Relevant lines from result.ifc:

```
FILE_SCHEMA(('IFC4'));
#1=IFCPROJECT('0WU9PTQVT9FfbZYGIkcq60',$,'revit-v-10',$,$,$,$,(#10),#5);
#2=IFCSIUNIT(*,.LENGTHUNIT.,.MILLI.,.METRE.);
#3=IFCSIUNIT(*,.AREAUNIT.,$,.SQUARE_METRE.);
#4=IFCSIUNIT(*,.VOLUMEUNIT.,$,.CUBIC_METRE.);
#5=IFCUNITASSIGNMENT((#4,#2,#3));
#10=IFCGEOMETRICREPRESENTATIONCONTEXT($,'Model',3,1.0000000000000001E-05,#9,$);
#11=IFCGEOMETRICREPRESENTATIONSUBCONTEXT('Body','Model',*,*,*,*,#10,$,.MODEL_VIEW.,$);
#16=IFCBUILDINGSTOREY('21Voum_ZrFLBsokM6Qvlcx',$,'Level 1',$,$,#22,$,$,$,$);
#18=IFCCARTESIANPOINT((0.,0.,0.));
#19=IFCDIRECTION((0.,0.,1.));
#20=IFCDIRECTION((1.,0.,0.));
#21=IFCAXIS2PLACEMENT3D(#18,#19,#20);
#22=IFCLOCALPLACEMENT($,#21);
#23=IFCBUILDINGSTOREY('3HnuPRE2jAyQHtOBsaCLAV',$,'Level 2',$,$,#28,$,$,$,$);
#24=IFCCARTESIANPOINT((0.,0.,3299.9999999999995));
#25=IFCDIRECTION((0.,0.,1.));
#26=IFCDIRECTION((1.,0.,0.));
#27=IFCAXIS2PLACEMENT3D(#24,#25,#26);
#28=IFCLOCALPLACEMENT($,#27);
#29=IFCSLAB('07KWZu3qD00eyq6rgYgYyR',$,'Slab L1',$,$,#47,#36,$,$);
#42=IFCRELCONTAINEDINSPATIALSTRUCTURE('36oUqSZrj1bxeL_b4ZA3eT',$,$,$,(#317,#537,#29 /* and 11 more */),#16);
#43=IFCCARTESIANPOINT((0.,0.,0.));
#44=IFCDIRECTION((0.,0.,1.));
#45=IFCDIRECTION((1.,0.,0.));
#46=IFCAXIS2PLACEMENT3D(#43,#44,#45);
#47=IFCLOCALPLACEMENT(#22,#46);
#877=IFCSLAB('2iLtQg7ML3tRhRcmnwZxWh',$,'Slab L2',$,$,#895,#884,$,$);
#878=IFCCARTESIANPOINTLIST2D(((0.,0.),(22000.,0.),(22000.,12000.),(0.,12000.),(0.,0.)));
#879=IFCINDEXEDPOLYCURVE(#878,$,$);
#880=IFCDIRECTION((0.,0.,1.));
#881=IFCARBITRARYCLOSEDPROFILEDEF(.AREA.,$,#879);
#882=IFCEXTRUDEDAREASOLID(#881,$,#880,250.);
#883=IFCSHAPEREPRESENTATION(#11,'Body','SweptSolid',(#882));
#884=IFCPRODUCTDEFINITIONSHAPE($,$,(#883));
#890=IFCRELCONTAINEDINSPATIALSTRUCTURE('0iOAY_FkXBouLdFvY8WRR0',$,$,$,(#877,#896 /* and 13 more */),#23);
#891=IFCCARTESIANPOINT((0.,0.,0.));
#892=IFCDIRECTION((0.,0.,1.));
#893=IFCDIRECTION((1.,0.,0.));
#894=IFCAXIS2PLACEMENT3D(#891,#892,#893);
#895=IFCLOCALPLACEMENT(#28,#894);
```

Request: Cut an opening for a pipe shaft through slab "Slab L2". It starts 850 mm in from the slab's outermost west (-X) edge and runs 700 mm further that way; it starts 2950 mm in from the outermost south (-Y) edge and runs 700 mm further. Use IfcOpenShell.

```python
import numpy as np
import ifcopenshell
import ifcopenshell.api.feature
import ifcopenshell.api.geometry
import ifcopenshell.api.root
import ifcopenshell.geom
import ifcopenshell.util.placement
import ifcopenshell.util.representation
import ifcopenshell.util.shape
import ifcopenshell.util.unit

model = ifcopenshell.open("result.ifc")
unit_scale = ifcopenshell.util.unit.calculate_unit_scale(model)
settings = ifcopenshell.geom.settings()


def volume(element):
    """Net volume in cubic metres, openings subtracted."""
    shape = ifcopenshell.geom.create_shape(settings, element)
    return ifcopenshell.util.shape.get_volume(shape.geometry)


slab = model.by_guid("2iLtQg7ML3tRhRcmnwZxWh")
before = volume(slab)

# Extent in the slab's own axes, in metres. The edges named are its -X and -Y sides.
slab_shape = ifcopenshell.geom.create_shape(settings, slab)
vertices = ifcopenshell.util.shape.get_vertices(slab_shape.geometry)
x_min, y_min, bottom = vertices.min(axis=0)
top = vertices[:, 2].max()

opening = ifcopenshell.api.root.create_entity(model, ifc_class="IfcOpeningElement", name="Pipe shaft opening", predefined_type="OPENING")
context = ifcopenshell.util.representation.get_context(model, "Model", "Body", "MODEL_VIEW")
width, depth = 0.7, 0.7
outline = [(0.0, 0.0), (width, 0.0), (width, depth), (0.0, depth), (0.0, 0.0)]
# Overshoot both faces by 50 mm so the cut is clean.
shape = ifcopenshell.api.geometry.add_slab_representation(
    model, context=context, depth=top - bottom + 0.1, polyline=outline
)
ifcopenshell.api.geometry.assign_representation(model, product=opening, representation=shape)

matrix = ifcopenshell.util.placement.get_local_placement(slab.ObjectPlacement)
matrix[:, 3] = matrix @ np.append(np.array([x_min + 0.85, y_min + 2.95, bottom - 0.05]) / unit_scale, 1.0)
ifcopenshell.api.geometry.edit_object_placement(model, product=opening, matrix=matrix, is_si=False)
ifcopenshell.api.feature.add_feature(model, feature=opening, element=slab)

after = volume(slab)

print(f"slab volume {before:.3f} -> {after:.3f} m3")

model.write("result_v2.ifc")
```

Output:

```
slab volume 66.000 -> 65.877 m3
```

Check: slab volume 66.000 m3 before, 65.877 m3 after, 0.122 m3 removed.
